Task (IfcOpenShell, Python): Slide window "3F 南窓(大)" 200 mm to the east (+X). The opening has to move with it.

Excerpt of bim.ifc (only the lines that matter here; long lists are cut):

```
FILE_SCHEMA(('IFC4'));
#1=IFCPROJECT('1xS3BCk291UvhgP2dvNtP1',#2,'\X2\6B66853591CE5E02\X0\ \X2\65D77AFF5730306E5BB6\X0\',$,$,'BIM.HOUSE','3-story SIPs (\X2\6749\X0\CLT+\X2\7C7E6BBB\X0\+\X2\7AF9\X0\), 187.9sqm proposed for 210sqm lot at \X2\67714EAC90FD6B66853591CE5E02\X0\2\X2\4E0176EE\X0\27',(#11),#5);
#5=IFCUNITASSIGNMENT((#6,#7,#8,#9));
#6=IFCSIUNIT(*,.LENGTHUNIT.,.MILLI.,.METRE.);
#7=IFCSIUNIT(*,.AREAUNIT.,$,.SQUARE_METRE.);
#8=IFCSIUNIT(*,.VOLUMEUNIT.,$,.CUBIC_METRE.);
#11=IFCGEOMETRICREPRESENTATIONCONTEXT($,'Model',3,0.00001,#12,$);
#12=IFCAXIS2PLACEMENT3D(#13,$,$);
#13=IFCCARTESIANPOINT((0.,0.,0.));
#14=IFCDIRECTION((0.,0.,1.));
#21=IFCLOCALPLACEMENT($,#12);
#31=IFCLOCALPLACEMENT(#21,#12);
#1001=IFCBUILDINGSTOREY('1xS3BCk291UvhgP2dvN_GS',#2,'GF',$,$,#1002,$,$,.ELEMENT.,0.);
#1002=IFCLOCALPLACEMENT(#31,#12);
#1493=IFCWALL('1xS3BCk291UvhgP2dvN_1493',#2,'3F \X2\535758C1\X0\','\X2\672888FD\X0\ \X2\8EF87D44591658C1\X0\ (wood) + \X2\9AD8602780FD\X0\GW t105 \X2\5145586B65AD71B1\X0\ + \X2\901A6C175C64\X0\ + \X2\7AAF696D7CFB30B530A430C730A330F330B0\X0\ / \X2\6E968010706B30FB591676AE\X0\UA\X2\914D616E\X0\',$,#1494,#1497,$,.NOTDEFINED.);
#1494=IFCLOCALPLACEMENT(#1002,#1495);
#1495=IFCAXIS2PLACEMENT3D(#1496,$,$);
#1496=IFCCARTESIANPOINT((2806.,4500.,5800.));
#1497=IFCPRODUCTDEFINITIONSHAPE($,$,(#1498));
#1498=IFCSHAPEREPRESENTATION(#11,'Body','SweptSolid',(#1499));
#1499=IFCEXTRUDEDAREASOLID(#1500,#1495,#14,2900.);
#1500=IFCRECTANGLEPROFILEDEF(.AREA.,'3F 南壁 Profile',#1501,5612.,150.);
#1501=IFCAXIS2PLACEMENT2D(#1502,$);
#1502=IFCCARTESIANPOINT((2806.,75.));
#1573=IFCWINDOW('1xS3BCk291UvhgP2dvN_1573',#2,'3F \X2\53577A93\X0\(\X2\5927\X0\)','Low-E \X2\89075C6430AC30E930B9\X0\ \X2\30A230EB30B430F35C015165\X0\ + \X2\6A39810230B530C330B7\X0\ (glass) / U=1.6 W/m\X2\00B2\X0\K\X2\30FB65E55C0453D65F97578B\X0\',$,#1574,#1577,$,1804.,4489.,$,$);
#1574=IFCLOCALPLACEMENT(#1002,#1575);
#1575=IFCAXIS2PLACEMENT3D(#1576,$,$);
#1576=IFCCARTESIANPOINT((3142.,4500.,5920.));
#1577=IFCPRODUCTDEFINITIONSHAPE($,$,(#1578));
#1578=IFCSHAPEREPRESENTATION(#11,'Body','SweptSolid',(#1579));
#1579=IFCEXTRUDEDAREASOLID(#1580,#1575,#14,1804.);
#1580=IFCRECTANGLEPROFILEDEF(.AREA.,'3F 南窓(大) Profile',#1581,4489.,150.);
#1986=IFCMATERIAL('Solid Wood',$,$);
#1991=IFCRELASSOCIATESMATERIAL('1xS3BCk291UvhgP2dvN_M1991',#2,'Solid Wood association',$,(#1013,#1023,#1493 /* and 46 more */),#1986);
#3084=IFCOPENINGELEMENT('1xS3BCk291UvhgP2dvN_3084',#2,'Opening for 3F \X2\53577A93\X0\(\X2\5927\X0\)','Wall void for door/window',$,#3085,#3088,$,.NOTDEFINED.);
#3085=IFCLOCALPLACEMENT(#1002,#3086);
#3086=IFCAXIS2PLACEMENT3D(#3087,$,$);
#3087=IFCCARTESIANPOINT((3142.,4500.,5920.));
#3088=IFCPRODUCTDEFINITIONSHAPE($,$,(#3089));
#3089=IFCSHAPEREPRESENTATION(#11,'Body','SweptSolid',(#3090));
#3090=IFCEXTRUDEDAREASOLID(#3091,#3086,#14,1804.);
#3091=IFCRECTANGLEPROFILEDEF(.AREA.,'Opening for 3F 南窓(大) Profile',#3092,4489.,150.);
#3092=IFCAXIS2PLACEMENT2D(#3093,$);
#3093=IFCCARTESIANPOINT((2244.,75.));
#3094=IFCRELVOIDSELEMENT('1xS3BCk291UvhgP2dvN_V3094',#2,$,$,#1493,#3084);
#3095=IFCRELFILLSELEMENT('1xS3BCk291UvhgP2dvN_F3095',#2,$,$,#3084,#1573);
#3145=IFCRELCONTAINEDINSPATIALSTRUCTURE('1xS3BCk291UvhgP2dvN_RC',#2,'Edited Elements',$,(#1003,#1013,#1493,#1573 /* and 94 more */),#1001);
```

```python
import ifcopenshell
import ifcopenshell.api.geometry
import ifcopenshell.util.placement

model = ifcopenshell.open("bim.ifc")

window = model.by_guid("1xS3BCk291UvhgP2dvN_1573")
opening = window.FillsVoids[0].RelatingOpeningElement
wall = opening.VoidsElements[0].RelatingBuildingElement

wall_matrix = ifcopenshell.util.placement.get_local_placement(wall.ObjectPlacement)
shift = wall_matrix[:3, 0] * 200.0
before = ifcopenshell.util.placement.get_local_placement(window.ObjectPlacement)[:3, 3].copy()

# The window is not placed relative to its opening, so move both.
for product in (opening, window):
    matrix = ifcopenshell.util.placement.get_local_placement(product.ObjectPlacement)
    matrix[:3, 3] += shift
    ifcopenshell.api.geometry.edit_object_placement(model, product=product, matrix=matrix, is_si=False)

after = ifcopenshell.util.placement.get_local_placement(window.ObjectPlacement)[:3, 3]
print("window moved by", (after - before).round(3) + 0.0)

model.write("bim_updated.ifc")
```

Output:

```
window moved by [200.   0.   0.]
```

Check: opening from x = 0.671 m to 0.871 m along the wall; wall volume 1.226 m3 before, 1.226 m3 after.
